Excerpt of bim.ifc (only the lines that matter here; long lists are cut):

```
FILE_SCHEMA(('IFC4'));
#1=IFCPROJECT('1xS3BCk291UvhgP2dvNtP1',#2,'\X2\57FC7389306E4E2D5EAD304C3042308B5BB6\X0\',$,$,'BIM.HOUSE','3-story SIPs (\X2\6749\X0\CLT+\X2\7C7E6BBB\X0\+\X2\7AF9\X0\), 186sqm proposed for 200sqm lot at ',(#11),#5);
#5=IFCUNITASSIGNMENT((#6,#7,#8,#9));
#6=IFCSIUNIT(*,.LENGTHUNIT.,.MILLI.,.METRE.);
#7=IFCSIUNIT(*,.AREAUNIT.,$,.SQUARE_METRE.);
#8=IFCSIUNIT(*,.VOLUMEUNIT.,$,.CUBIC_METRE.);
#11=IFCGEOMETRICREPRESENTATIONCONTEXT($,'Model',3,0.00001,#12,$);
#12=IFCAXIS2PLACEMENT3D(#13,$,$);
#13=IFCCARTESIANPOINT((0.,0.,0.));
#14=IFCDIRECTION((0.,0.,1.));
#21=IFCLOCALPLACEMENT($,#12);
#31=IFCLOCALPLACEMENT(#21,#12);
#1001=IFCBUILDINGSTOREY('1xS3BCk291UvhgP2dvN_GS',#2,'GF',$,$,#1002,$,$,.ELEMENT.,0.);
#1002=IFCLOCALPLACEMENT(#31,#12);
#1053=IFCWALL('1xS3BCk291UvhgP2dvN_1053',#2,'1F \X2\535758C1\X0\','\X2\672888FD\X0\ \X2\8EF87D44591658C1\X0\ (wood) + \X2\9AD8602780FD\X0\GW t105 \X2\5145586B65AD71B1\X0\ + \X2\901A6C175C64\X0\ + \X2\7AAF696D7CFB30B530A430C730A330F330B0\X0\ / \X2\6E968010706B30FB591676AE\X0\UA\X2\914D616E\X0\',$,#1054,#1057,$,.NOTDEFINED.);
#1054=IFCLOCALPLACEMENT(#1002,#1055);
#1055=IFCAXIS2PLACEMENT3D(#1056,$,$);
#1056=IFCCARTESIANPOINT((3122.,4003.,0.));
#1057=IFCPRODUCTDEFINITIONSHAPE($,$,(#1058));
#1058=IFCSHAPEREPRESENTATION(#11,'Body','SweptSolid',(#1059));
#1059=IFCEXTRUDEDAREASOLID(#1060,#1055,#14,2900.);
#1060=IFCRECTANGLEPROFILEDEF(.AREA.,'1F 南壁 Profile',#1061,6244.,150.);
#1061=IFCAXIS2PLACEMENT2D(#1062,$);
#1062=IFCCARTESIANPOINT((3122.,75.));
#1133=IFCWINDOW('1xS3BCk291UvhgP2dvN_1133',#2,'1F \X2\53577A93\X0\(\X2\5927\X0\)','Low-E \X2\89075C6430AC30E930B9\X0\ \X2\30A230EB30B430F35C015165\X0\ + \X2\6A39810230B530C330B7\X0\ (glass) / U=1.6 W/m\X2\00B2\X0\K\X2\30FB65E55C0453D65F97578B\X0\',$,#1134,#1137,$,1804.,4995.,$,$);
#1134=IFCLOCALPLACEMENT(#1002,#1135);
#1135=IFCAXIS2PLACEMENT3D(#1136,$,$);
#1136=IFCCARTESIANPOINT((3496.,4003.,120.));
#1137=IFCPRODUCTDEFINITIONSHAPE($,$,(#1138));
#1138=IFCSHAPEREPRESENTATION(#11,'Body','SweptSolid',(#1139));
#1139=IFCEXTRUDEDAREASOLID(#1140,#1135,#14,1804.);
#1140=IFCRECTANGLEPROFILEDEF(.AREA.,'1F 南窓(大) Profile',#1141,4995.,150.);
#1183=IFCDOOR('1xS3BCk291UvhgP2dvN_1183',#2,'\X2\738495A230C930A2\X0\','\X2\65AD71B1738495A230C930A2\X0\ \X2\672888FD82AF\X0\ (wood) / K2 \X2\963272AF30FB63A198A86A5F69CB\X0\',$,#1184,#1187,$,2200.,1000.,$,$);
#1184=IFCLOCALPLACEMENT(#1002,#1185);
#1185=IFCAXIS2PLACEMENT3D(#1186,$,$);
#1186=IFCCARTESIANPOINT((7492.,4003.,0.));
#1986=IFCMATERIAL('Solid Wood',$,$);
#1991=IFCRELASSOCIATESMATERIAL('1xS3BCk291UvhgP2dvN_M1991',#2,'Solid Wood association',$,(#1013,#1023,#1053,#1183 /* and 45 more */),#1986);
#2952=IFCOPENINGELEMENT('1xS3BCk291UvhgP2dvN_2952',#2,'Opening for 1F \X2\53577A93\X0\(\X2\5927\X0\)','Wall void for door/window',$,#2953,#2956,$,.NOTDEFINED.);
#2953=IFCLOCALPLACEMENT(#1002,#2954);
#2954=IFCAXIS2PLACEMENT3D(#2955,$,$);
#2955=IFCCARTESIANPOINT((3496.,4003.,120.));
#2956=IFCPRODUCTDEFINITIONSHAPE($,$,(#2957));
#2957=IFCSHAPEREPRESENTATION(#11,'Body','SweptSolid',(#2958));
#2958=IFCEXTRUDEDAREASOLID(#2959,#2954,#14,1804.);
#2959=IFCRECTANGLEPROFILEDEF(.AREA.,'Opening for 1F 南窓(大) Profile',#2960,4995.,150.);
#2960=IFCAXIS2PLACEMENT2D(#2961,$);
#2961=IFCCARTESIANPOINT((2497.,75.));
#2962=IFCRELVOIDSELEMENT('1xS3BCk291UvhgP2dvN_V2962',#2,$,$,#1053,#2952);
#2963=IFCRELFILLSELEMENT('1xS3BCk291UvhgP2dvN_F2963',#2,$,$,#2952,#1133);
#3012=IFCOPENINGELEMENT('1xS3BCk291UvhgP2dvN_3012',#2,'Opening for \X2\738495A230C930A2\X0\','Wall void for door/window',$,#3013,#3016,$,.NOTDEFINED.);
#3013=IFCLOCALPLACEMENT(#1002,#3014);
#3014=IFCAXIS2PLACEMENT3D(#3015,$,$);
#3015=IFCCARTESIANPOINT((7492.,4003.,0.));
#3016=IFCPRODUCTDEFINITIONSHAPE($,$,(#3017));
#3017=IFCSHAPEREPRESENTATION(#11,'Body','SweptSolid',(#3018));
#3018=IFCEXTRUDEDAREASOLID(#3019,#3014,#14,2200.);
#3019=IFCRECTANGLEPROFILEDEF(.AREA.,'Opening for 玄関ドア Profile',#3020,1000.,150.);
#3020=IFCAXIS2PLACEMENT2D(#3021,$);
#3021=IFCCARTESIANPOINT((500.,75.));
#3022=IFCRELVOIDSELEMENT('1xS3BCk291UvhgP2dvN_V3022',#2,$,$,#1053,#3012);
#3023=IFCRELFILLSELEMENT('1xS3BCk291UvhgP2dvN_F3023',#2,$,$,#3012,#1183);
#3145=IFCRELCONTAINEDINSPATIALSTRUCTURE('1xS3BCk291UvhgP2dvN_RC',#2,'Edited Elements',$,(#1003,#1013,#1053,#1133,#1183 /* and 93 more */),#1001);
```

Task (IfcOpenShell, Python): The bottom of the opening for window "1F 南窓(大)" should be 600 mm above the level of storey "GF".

```python
import numpy as np
import ifcopenshell
import ifcopenshell.api.geometry
import ifcopenshell.geom
import ifcopenshell.util.element
import ifcopenshell.util.placement
import ifcopenshell.util.shape
import ifcopenshell.util.unit

model = ifcopenshell.open("bim.ifc")
unit_scale = ifcopenshell.util.unit.calculate_unit_scale(model)

window = model.by_guid("1xS3BCk291UvhgP2dvN_1133")
opening = window.FillsVoids[0].RelatingOpeningElement
storey = ifcopenshell.util.element.get_container(window, ifc_class="IfcBuildingStorey")
level = ifcopenshell.util.placement.get_local_placement(storey.ObjectPlacement)[2, 3]

# The opening's origin need not be at the sill, so measure its lowest point.
shape = ifcopenshell.geom.create_shape(ifcopenshell.geom.settings(), opening)
bottom = ifcopenshell.util.shape.get_shape_bottom_elevation(shape, shape.geometry) / unit_scale
dz = level + 600.0 - bottom

shift = np.array([0.0, 0.0, dz])
# The window is not placed relative to its opening, so move both.
for product in (opening, window):
    matrix = ifcopenshell.util.placement.get_local_placement(product.ObjectPlacement)
    matrix[:3, 3] += shift
    ifcopenshell.api.geometry.edit_object_placement(model, product=product, matrix=matrix, is_si=False)

print(f"moved by {dz * unit_scale:+.3f} m")

model.write("bim-out.ifc")
```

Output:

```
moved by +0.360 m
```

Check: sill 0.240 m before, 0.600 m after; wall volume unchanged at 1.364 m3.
